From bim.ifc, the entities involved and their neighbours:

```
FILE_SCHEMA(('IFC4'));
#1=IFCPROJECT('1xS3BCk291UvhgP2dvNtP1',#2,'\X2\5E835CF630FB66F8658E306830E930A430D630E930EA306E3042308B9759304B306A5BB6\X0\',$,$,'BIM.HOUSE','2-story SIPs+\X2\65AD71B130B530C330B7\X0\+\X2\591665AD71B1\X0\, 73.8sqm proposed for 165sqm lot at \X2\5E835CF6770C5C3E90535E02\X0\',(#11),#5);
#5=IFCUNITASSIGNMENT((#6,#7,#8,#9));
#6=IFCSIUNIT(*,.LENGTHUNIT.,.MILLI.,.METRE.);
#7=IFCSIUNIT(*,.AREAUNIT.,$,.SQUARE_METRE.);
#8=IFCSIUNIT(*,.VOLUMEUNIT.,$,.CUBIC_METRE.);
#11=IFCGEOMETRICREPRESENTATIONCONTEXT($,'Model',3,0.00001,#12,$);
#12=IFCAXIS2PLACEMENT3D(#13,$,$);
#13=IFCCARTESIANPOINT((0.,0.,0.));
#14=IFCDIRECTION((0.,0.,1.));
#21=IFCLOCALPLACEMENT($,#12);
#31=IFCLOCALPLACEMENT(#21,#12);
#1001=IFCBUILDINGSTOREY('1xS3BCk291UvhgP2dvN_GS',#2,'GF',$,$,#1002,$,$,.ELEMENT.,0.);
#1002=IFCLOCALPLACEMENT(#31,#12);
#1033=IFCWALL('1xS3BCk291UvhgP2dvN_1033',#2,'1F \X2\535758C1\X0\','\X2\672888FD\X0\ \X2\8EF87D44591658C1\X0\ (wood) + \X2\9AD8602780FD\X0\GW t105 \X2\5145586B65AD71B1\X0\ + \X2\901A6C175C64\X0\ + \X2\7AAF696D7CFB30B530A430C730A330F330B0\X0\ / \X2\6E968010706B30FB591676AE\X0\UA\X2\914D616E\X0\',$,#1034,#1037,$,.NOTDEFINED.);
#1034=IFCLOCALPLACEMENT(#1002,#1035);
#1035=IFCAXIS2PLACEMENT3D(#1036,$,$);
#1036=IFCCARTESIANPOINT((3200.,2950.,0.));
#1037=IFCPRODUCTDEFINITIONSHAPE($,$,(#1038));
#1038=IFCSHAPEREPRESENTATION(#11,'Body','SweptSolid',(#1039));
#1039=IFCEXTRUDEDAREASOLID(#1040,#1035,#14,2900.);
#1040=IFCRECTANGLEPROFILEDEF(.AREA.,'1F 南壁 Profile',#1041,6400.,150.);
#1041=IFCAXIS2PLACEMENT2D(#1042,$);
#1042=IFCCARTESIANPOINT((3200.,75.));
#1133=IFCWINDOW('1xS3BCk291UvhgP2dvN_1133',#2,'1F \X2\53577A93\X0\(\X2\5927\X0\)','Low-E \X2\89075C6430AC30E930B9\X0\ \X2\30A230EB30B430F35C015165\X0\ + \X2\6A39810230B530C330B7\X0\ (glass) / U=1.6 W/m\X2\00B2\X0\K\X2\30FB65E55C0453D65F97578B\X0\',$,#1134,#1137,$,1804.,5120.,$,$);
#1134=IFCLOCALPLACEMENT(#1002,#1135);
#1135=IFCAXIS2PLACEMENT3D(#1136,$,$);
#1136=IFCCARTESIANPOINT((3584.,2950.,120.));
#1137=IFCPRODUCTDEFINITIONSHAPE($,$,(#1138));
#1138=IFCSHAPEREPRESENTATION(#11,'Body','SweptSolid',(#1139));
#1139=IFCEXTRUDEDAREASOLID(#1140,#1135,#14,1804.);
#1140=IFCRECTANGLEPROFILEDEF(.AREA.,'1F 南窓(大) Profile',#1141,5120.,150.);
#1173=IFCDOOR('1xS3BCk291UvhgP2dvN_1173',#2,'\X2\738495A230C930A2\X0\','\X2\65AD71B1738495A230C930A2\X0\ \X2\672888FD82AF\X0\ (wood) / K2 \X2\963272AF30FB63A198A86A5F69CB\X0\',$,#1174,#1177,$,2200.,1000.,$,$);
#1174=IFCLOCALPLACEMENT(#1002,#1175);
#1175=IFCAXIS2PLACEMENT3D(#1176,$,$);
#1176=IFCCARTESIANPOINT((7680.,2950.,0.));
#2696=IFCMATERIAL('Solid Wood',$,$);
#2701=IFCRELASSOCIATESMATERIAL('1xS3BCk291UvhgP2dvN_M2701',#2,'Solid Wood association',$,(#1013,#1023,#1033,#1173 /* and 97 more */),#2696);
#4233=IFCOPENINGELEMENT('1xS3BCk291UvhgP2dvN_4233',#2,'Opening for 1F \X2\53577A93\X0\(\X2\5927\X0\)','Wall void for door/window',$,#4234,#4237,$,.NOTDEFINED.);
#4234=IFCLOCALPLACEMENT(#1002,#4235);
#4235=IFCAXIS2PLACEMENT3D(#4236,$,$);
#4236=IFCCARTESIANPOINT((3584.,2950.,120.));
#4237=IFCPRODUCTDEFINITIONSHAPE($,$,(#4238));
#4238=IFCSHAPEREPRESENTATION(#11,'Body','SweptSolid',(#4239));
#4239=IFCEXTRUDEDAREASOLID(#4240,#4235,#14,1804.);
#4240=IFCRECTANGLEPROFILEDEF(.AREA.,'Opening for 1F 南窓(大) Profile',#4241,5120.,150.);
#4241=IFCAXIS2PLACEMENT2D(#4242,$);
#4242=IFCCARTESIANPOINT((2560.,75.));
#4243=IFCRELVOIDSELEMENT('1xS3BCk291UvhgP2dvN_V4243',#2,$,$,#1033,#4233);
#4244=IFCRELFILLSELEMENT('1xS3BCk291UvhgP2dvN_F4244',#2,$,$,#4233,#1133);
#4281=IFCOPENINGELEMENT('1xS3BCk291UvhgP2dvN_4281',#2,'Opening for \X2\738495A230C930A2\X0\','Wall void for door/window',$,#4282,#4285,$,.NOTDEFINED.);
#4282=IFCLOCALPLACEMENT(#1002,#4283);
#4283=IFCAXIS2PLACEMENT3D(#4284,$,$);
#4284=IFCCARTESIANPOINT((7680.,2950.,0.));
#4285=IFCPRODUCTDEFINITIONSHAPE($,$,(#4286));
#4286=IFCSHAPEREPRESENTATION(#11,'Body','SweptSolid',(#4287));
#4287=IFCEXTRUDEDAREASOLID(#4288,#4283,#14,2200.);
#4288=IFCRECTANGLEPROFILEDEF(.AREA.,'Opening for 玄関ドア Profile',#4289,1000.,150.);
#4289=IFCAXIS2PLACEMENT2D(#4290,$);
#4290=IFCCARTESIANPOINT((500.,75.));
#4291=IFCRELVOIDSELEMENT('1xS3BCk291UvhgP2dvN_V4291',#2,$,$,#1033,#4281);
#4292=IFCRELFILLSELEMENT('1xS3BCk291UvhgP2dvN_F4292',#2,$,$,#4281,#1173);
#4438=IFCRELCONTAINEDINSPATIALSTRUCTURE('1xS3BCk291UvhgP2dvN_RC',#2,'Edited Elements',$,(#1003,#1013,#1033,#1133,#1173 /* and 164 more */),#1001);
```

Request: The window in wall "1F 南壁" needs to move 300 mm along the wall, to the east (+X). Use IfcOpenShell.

```python
import ifcopenshell
import ifcopenshell.api.geometry
import ifcopenshell.util.placement
import ifcopenshell.util.unit

model = ifcopenshell.open("bim.ifc")
unit_scale = ifcopenshell.util.unit.calculate_unit_scale(model)

window = model.by_guid("1xS3BCk291UvhgP2dvN_1133")
opening = window.FillsVoids[0].RelatingOpeningElement
wall = opening.VoidsElements[0].RelatingBuildingElement

wall_matrix = ifcopenshell.util.placement.get_local_placement(wall.ObjectPlacement)
shift = wall_matrix[:3, 0] * 0.3 / unit_scale
before = ifcopenshell.util.placement.get_local_placement(window.ObjectPlacement)[:3, 3].copy()

# The window is not placed relative to its opening, so move both.
for product in (opening, window):
    matrix = ifcopenshell.util.placement.get_local_placement(product.ObjectPlacement)
    matrix[:3, 3] += shift
    ifcopenshell.api.geometry.edit_object_placement(model, product=product, matrix=matrix, is_si=False)

after = ifcopenshell.util.placement.get_local_placement(window.ObjectPlacement)[:3, 3]
print("window moved by", (after - before).round(3) + 0.0)

model.write("bim_edited.ifc")
```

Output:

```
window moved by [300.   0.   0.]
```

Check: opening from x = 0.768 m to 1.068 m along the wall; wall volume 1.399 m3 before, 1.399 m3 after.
